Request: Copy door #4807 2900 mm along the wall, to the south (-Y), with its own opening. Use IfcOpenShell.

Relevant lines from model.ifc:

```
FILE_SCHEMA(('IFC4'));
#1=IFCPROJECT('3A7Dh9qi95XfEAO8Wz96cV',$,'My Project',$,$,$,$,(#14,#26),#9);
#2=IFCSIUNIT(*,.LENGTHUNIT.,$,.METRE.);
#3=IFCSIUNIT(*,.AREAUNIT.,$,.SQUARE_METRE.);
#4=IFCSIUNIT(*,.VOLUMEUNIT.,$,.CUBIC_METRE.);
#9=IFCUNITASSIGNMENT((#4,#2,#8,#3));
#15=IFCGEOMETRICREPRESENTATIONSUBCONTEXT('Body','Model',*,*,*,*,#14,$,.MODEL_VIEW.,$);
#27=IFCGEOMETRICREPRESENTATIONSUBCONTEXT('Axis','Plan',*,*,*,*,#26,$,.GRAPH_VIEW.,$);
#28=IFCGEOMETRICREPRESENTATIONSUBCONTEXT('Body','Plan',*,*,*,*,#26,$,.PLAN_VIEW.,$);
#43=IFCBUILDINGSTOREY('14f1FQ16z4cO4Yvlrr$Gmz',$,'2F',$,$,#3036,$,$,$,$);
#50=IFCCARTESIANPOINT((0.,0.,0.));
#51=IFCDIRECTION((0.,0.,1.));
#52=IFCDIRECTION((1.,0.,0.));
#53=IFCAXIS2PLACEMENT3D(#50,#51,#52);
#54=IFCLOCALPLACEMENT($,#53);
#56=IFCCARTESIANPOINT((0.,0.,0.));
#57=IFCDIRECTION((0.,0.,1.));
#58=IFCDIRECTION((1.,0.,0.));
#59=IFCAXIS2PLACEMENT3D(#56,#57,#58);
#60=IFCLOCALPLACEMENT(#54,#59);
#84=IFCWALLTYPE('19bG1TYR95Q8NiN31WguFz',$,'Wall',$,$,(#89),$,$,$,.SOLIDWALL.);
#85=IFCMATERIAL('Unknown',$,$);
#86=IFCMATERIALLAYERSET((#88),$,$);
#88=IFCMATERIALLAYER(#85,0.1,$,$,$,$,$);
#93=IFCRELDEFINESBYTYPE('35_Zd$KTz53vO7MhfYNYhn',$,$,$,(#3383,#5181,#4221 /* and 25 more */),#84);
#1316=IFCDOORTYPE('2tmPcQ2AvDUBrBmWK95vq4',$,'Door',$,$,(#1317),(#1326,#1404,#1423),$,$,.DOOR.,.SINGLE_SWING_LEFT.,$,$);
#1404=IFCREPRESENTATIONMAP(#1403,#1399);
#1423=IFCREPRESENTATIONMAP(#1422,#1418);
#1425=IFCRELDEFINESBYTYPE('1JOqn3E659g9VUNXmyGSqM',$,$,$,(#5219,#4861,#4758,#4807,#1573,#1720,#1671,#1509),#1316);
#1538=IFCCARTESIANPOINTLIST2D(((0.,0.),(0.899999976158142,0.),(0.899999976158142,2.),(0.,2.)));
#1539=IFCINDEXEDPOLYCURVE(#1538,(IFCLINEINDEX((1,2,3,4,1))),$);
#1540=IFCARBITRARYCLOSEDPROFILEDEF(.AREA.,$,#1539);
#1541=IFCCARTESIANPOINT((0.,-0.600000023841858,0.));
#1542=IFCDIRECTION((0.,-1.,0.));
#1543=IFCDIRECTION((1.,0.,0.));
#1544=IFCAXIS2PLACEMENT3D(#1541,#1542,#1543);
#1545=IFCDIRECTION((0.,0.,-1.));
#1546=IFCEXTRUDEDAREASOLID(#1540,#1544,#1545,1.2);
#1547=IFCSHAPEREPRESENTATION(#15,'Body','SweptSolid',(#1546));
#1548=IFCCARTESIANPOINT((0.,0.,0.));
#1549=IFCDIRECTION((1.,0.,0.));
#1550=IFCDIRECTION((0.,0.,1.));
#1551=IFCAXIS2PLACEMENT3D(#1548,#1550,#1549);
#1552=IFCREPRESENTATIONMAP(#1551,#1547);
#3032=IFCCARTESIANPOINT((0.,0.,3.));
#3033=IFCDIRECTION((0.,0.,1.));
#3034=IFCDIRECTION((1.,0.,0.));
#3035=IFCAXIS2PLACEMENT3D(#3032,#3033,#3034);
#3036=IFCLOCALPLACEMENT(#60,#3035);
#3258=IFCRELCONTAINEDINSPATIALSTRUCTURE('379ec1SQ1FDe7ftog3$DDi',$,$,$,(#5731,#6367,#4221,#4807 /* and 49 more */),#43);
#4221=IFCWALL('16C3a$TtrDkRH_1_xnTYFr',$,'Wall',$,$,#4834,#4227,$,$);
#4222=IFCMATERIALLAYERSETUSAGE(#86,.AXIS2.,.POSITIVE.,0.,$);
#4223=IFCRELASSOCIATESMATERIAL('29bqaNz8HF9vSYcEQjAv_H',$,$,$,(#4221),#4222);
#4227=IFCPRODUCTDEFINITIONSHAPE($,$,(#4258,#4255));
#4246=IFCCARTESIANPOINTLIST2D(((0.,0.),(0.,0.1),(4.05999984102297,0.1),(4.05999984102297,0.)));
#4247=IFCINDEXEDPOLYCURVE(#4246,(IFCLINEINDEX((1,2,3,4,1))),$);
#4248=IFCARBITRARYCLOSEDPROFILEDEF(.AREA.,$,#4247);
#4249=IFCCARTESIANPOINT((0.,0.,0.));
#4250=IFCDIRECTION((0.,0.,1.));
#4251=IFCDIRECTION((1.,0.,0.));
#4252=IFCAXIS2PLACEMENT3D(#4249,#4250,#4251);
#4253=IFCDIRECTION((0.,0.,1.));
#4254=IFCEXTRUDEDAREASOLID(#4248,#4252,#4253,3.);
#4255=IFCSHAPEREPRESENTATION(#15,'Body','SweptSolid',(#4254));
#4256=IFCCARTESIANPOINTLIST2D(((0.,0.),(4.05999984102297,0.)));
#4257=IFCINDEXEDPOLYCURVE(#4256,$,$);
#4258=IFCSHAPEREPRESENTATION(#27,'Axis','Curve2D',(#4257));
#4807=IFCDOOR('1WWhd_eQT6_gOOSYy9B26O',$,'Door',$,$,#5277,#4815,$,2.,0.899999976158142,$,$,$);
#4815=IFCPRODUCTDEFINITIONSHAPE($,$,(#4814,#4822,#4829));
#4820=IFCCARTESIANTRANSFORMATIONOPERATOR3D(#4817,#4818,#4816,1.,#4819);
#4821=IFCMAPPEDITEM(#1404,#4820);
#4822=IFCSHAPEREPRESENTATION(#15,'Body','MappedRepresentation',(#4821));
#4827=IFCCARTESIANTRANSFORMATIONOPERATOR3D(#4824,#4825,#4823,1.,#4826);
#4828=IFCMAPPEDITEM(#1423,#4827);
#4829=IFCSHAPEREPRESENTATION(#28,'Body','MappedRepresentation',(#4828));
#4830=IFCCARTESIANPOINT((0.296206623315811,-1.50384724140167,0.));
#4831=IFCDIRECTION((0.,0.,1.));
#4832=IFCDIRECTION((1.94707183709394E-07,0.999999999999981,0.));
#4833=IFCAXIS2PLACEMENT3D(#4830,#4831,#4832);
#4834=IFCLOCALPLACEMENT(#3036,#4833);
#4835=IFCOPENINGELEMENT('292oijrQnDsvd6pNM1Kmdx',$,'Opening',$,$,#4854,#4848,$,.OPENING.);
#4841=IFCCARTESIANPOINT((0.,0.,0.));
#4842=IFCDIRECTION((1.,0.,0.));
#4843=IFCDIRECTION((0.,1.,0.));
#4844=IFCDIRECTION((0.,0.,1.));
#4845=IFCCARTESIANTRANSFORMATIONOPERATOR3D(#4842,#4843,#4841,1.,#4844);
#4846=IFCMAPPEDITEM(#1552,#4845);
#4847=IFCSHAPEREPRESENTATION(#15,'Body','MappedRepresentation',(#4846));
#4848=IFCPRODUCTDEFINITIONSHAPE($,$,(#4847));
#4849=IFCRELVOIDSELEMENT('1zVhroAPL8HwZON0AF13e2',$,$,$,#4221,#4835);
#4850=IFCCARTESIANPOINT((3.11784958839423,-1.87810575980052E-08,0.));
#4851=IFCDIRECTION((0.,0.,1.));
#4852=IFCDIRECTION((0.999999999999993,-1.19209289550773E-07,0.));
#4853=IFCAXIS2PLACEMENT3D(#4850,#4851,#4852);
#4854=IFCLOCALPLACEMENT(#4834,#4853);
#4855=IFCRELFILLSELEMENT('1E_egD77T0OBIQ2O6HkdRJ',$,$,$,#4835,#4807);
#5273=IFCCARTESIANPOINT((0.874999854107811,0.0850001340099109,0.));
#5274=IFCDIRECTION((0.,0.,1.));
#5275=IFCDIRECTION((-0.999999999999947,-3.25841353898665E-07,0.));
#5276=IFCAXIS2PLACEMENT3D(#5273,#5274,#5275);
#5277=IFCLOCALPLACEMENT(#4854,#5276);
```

```python
import ifcopenshell
import ifcopenshell.api.feature
import ifcopenshell.api.geometry
import ifcopenshell.api.root
import ifcopenshell.geom
import ifcopenshell.util.element
import ifcopenshell.util.placement
import ifcopenshell.util.shape

model = ifcopenshell.open("model.ifc")
settings = ifcopenshell.geom.settings()


def volume(element):
    """Net volume in cubic metres, openings subtracted."""
    shape = ifcopenshell.geom.create_shape(settings, element)
    return ifcopenshell.util.shape.get_volume(shape.geometry)


door = model.by_id(4807)
opening = door.FillsVoids[0].RelatingOpeningElement
wall = opening.VoidsElements[0].RelatingBuildingElement
before = volume(wall)
shift = ifcopenshell.util.placement.get_local_placement(wall.ObjectPlacement)[:3, 0] * -2.9

# copy_class copies the void relationship, type, container and properties, but no geometry.
new_opening = ifcopenshell.api.root.copy_class(model, product=opening)
new_opening.Representation = ifcopenshell.util.element.copy_deep(
    model, opening.Representation, exclude=["IfcGeometricRepresentationContext", "IfcRepresentationMap"]
)
new_door = ifcopenshell.api.root.copy_class(model, product=door)
new_door.Representation = ifcopenshell.util.element.copy_deep(
    model, door.Representation, exclude=["IfcGeometricRepresentationContext", "IfcRepresentationMap"]
)
ifcopenshell.api.feature.add_filling(model, opening=new_opening, element=new_door)

for old, new in ((opening, new_opening), (door, new_door)):
    matrix = ifcopenshell.util.placement.get_local_placement(old.ObjectPlacement)
    matrix[:3, 3] += shift
    ifcopenshell.api.geometry.edit_object_placement(model, product=new, matrix=matrix, is_si=False)

after = volume(wall)

print(f"wall volume {before:.3f} -> {after:.3f} m3")

model.write("model_v2.ifc")
```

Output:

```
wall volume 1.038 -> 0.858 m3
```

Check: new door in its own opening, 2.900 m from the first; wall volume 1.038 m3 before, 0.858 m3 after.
